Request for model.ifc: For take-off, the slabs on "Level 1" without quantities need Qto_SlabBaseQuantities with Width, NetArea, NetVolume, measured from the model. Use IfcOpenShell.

First a look at what the model holds.

```python
import ifcopenshell
import ifcopenshell.util.element
import ifcopenshell.util.unit

model = ifcopenshell.open("model.ifc")
print(model.schema)
for unit_type in ("LENGTHUNIT", "AREAUNIT", "VOLUMEUNIT"):
    print(unit_type, ifcopenshell.util.unit.calculate_unit_scale(model, unit_type))
storey = next(s for s in model.by_type("IfcBuildingStorey") if s.Name == "Level 1")
slabs = [e for e in ifcopenshell.util.element.get_decomposition(storey) if e.is_a("IfcSlab")]
for e in sorted(slabs, key=lambda e: e.id()):
    print(e.id(), e.is_a(), e.Name, list(ifcopenshell.util.element.get_psets(e, qtos_only=True)), sep=" | ")
```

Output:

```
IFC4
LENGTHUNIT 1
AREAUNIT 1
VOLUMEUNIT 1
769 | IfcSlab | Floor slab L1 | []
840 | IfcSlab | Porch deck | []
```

```python
import ifcopenshell
import ifcopenshell.api.pset
import ifcopenshell.geom
import ifcopenshell.util.element
import ifcopenshell.util.shape
import ifcopenshell.util.unit

model = ifcopenshell.open("model.ifc")
unit_scale = ifcopenshell.util.unit.calculate_unit_scale(model)
area_scale = ifcopenshell.util.unit.calculate_unit_scale(model, "AREAUNIT")
volume_scale = ifcopenshell.util.unit.calculate_unit_scale(model, "VOLUMEUNIT")
settings = ifcopenshell.geom.settings()

storey = next(s for s in model.by_type("IfcBuildingStorey") if s.Name == "Level 1")
slabs = [e for e in ifcopenshell.util.element.get_decomposition(storey) if e.is_a("IfcSlab")]

for e in sorted(slabs, key=lambda e: e.id()):
    if ifcopenshell.util.element.get_psets(e, qtos_only=True, should_inherit=False):
        continue
    # Geometry comes back in metres, in the element's own axes.
    shape = ifcopenshell.geom.create_shape(settings, e)
    values = {
        "Width": ifcopenshell.util.shape.get_z(shape.geometry) / unit_scale,
        "NetArea": ifcopenshell.util.shape.get_footprint_area(shape.geometry) / area_scale,
        "NetVolume": ifcopenshell.util.shape.get_volume(shape.geometry) / volume_scale,
    }
    qto = ifcopenshell.api.pset.add_qto(model, product=e, name="Qto_SlabBaseQuantities")
    ifcopenshell.api.pset.edit_qto(model, qto=qto, properties=values)
    print(e.id(), {k: round(v, 3) for k, v in values.items()})

model.write("model_updated.ifc")
```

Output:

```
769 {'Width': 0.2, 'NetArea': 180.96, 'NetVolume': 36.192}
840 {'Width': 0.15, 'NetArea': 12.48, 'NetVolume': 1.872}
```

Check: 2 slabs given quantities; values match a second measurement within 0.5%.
